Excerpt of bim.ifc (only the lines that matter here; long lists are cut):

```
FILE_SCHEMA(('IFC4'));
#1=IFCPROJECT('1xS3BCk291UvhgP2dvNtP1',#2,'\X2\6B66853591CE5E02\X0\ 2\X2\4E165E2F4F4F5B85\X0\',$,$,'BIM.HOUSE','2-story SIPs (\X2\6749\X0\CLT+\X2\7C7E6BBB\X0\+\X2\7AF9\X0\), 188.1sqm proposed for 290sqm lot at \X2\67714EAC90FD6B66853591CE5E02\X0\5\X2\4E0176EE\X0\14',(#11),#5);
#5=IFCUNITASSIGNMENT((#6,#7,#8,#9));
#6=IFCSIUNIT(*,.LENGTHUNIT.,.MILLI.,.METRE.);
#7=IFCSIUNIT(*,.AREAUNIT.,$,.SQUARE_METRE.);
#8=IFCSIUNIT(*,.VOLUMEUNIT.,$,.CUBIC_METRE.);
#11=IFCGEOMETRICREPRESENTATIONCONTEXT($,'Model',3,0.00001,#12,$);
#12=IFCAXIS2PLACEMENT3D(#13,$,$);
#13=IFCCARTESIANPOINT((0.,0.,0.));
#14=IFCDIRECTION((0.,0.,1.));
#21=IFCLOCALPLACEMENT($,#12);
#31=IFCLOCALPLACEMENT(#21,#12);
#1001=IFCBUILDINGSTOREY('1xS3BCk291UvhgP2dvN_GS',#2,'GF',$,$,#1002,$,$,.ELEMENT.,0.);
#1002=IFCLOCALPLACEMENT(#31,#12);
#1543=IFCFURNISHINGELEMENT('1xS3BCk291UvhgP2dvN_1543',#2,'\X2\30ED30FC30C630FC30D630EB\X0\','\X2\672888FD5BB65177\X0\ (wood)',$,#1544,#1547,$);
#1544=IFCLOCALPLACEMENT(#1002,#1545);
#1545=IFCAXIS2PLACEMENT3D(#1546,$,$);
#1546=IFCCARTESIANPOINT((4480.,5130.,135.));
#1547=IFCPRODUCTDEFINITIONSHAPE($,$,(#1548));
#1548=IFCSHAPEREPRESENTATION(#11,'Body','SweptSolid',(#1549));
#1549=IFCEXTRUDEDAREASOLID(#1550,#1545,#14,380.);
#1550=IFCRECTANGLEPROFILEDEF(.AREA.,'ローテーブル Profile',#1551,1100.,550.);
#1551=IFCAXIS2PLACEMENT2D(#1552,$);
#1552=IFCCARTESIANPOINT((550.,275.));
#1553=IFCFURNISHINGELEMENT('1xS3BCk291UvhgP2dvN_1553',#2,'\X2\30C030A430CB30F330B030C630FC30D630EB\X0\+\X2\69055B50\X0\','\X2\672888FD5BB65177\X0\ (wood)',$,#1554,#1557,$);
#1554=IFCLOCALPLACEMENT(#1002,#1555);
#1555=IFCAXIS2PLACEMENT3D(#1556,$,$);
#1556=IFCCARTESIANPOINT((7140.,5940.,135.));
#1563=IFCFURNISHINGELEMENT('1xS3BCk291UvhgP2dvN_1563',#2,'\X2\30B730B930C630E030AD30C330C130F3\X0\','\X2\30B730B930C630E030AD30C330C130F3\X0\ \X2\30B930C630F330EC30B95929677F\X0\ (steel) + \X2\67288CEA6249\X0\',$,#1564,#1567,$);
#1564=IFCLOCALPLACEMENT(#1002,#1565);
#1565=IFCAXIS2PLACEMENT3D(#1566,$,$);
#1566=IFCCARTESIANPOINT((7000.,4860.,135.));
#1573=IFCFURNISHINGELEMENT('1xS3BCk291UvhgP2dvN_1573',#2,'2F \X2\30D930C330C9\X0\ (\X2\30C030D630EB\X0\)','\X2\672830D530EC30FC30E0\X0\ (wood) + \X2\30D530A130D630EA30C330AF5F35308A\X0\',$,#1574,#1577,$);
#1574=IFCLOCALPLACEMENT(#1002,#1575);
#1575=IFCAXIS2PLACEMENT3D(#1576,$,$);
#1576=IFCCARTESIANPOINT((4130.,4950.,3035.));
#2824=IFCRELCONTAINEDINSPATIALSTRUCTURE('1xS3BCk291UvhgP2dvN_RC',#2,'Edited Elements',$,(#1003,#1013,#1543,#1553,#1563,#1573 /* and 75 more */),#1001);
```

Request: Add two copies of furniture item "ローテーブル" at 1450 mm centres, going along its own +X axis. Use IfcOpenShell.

```python
import ifcopenshell
import ifcopenshell.api.geometry
import ifcopenshell.api.root
import ifcopenshell.util.element
import ifcopenshell.util.placement
import ifcopenshell.util.unit

model = ifcopenshell.open("bim.ifc")
unit_scale = ifcopenshell.util.unit.calculate_unit_scale(model)


def reuse_history(source, copy):
    """copy_class also copies each property set's owner history, people and application; keep the originals."""
    for rel in copy.IsDefinedBy:
        if rel.is_a("IfcRelDefinesByProperties") and (history := rel.RelatingPropertyDefinition.OwnerHistory):
            rel.RelatingPropertyDefinition.OwnerHistory = source.OwnerHistory
            ifcopenshell.util.element.remove_deep2(model, history)


source = model.by_guid("1xS3BCk291UvhgP2dvN_1543")
base = ifcopenshell.util.placement.get_local_placement(source.ObjectPlacement)
step = base[:3, 0] * 1.45 / unit_scale

for i in range(1, 3):
    copy = ifcopenshell.api.root.copy_class(model, product=source)
    copy.Representation = ifcopenshell.util.element.copy_deep(
        model, source.Representation, exclude=["IfcGeometricRepresentationContext", "IfcRepresentationMap"]
    )
    reuse_history(source, copy)
    matrix = base.copy()
    matrix[:3, 3] += i * step
    print("added at", matrix[:3, 3].round(3) + 0.0)
    ifcopenshell.api.geometry.edit_object_placement(model, product=copy, matrix=matrix, is_si=False)

model.write("bim_updated.ifc")
```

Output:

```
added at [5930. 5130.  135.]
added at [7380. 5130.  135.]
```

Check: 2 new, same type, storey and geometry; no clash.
